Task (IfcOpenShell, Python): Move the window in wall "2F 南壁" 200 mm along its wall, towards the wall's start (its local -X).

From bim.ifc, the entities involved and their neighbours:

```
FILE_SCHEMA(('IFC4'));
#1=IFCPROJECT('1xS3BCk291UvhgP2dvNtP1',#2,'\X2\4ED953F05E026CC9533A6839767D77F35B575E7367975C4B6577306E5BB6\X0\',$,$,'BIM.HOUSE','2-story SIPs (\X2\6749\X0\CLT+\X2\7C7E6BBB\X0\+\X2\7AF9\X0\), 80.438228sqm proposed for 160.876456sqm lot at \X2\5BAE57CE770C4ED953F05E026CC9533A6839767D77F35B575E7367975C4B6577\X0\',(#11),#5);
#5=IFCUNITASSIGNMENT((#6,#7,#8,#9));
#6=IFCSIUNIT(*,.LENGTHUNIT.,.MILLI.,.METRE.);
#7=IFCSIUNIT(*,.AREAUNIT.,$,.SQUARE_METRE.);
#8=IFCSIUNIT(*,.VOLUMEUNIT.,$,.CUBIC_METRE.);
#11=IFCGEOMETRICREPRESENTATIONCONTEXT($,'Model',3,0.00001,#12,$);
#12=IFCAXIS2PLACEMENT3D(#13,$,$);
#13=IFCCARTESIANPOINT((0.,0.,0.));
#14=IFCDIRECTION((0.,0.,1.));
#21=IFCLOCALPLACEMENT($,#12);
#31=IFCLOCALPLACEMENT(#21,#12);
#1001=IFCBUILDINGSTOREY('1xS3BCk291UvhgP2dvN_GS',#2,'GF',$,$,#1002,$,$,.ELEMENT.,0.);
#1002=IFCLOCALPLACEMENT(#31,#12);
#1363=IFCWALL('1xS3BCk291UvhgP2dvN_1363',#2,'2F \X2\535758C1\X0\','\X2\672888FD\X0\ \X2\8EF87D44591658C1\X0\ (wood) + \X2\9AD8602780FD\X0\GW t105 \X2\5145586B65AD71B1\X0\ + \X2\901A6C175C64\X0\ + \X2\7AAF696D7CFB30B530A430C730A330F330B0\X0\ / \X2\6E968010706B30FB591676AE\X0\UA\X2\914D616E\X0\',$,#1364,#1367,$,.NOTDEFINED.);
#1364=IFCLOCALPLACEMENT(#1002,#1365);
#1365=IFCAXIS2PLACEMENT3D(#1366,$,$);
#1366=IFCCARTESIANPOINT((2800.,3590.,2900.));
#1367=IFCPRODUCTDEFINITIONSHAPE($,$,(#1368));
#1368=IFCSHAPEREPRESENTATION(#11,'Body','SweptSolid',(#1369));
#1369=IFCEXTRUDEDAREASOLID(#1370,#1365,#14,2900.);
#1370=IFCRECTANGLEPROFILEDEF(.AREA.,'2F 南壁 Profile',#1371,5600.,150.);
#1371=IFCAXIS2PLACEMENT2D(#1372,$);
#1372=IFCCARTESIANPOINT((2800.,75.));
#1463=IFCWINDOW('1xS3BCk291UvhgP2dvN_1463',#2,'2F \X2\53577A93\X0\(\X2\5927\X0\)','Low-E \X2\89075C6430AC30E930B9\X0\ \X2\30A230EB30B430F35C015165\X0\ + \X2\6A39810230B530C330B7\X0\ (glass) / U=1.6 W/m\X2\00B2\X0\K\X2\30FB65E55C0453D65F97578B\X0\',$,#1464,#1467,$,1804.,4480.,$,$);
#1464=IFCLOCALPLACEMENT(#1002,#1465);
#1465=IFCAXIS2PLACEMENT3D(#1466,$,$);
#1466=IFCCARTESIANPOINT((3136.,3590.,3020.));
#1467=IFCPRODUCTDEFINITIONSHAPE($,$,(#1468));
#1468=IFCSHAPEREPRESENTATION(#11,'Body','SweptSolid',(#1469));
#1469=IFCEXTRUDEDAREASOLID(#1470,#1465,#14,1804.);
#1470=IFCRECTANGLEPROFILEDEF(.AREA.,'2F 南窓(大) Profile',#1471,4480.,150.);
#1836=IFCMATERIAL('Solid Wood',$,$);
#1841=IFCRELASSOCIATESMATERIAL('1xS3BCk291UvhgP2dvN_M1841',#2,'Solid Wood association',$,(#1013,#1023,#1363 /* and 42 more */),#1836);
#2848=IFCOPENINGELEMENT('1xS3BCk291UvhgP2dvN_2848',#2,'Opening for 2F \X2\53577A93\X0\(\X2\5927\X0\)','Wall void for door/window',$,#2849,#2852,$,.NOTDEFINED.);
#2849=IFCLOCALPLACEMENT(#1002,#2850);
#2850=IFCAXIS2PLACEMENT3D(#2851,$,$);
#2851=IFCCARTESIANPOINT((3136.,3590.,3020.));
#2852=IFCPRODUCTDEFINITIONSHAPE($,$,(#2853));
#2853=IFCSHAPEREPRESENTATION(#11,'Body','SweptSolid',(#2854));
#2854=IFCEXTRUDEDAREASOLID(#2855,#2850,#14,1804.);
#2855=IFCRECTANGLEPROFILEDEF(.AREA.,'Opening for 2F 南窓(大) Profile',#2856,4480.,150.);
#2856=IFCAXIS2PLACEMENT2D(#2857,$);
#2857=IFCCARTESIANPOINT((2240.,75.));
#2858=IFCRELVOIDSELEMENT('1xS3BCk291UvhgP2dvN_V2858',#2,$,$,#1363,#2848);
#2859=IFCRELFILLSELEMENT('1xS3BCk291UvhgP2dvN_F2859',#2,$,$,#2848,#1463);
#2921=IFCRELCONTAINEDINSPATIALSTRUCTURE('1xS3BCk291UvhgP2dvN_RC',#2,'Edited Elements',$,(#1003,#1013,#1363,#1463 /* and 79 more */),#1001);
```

```python
import ifcopenshell
import ifcopenshell.api.geometry
import ifcopenshell.util.placement
import ifcopenshell.util.unit

model = ifcopenshell.open("bim.ifc")
unit_scale = ifcopenshell.util.unit.calculate_unit_scale(model)

window = model.by_guid("1xS3BCk291UvhgP2dvN_1463")
opening = window.FillsVoids[0].RelatingOpeningElement
wall = opening.VoidsElements[0].RelatingBuildingElement

wall_matrix = ifcopenshell.util.placement.get_local_placement(wall.ObjectPlacement)
shift = wall_matrix[:3, 0] * -0.2 / unit_scale
before = ifcopenshell.util.placement.get_local_placement(window.ObjectPlacement)[:3, 3].copy()

# The window is not placed relative to its opening, so move both.
for product in (opening, window):
    matrix = ifcopenshell.util.placement.get_local_placement(product.ObjectPlacement)
    matrix[:3, 3] += shift
    ifcopenshell.api.geometry.edit_object_placement(model, product=product, matrix=matrix, is_si=False)

after = ifcopenshell.util.placement.get_local_placement(window.ObjectPlacement)[:3, 3]
print("window moved by", (after - before).round(3) + 0.0)

model.write("bim_rev.ifc")
```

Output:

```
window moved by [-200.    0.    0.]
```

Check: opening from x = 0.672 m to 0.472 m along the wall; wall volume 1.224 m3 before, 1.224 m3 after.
